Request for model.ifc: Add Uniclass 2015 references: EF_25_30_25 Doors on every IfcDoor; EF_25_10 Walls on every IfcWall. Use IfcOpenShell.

First a look at what the model holds.

```python
import ifcopenshell

model = ifcopenshell.open("model.ifc")
print(model.schema)
print("classifications:", [c.Name for c in model.by_type("IfcClassification")])
for ifc_class in ("IfcDoor", "IfcRoof", "IfcStair", "IfcWall", "IfcWindow"):
    print(ifc_class, len(model.by_type(ifc_class)))
```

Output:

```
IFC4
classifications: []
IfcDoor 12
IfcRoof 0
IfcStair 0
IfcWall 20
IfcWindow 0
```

```python
import ifcopenshell
import ifcopenshell.api.classification

model = ifcopenshell.open("model.ifc")

system = ifcopenshell.api.classification.add_classification(model, classification="Uniclass 2015")

codes = {
    "IfcDoor": ("EF_25_30_25", "Doors"),
    "IfcWall": ("EF_25_10", "Walls"),
}
for ifc_class, (code, name) in codes.items():
    products = model.by_type(ifc_class)
    ifcopenshell.api.classification.add_reference(
        model, products=products, classification=system, identification=code, name=name
    )
    print(code, len(products))

model.write("model_v2.ifc")
```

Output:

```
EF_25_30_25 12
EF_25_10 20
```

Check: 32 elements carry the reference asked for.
